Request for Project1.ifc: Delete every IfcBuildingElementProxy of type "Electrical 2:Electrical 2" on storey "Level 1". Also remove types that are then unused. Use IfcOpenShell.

First a look at what the model holds.

```python
import ifcopenshell
import ifcopenshell.util.element

model = ifcopenshell.open("Project1.ifc")
print(model.schema)
storey = next(s for s in model.by_type("IfcBuildingStorey") if s.Name == "Level 1")
proxies = [e for e in ifcopenshell.util.element.get_decomposition(storey) if e.is_a("IfcBuildingElementProxy")]
seen = {}
for e in proxies:
    element_type = ifcopenshell.util.element.get_type(e)
    name = element_type.Name if element_type not in (None, e) else None
    seen[name] = seen.get(name, 0) + 1
for name, count in sorted(seen.items(), key=str):
    print(count, "x", name)
```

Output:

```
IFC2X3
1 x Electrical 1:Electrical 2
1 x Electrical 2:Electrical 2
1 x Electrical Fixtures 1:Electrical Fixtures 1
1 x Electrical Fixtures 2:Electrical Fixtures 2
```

```python
import ifcopenshell
import ifcopenshell.api.root
import ifcopenshell.util.element

model = ifcopenshell.open("Project1.ifc")

storey = next(s for s in model.by_type("IfcBuildingStorey") if s.Name == "Level 1")
proxies = [e for e in ifcopenshell.util.element.get_decomposition(storey) if e.is_a("IfcBuildingElementProxy")]
targets = [e for e in proxies if (t := ifcopenshell.util.element.get_type(e)) not in (None, e) and t.Name == "Electrical 2:Electrical 2"]
types = {ifcopenshell.util.element.get_type(e) for e in targets} - {None, *targets}

for e in targets:
    ifcopenshell.api.root.remove_product(model, product=e)
print(len(targets), "removed")

unused = [t for t in types if not ifcopenshell.util.element.get_types(t)]
for t in unused:
    ifcopenshell.api.root.remove_product(model, product=t)
print(len(unused), "unused types removed")

model.write("Project1_edited.ifc")
```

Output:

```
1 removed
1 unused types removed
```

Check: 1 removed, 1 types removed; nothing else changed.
